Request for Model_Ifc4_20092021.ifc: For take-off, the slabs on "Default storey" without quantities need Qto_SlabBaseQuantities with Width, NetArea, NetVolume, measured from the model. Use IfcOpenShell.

First a look at what the model holds.

```python
import ifcopenshell
import ifcopenshell.util.element
import ifcopenshell.util.unit

model = ifcopenshell.open("Model_Ifc4_20092021.ifc")
print(model.schema)
for unit_type in ("LENGTHUNIT", "AREAUNIT", "VOLUMEUNIT"):
    print(unit_type, ifcopenshell.util.unit.calculate_unit_scale(model, unit_type))
storey = next(s for s in model.by_type("IfcBuildingStorey") if s.Name == "Default storey")
slabs = [e for e in ifcopenshell.util.element.get_decomposition(storey) if e.is_a("IfcSlab")]
for e in sorted(slabs, key=lambda e: e.id()):
    print(e.id(), e.is_a(), e.Name, list(ifcopenshell.util.element.get_psets(e, qtos_only=True)), sep=" | ")
```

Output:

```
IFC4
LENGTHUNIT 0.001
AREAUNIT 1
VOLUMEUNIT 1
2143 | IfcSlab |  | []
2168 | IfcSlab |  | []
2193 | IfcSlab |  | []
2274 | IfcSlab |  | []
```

```python
import ifcopenshell
import ifcopenshell.api.pset
import ifcopenshell.geom
import ifcopenshell.util.element
import ifcopenshell.util.shape
import ifcopenshell.util.unit

model = ifcopenshell.open("Model_Ifc4_20092021.ifc")
unit_scale = ifcopenshell.util.unit.calculate_unit_scale(model)
area_scale = ifcopenshell.util.unit.calculate_unit_scale(model, "AREAUNIT")
volume_scale = ifcopenshell.util.unit.calculate_unit_scale(model, "VOLUMEUNIT")
settings = ifcopenshell.geom.settings()

storey = next(s for s in model.by_type("IfcBuildingStorey") if s.Name == "Default storey")
slabs = [e for e in ifcopenshell.util.element.get_decomposition(storey) if e.is_a("IfcSlab")]

for e in sorted(slabs, key=lambda e: e.id()):
    if ifcopenshell.util.element.get_psets(e, qtos_only=True, should_inherit=False):
        continue
    # Geometry comes back in metres, in the element's own axes.
    shape = ifcopenshell.geom.create_shape(settings, e)
    values = {
        "Width": ifcopenshell.util.shape.get_z(shape.geometry) / unit_scale,
        "NetArea": ifcopenshell.util.shape.get_footprint_area(shape.geometry) / area_scale,
        "NetVolume": ifcopenshell.util.shape.get_volume(shape.geometry) / volume_scale,
    }
    qto = ifcopenshell.api.pset.add_qto(model, product=e, name="Qto_SlabBaseQuantities")
    ifcopenshell.api.pset.edit_qto(model, qto=qto, properties=values)
    print(e.id(), {k: round(v, 3) for k, v in values.items()})

model.write("Model_Ifc4_20092021_edited.ifc")
```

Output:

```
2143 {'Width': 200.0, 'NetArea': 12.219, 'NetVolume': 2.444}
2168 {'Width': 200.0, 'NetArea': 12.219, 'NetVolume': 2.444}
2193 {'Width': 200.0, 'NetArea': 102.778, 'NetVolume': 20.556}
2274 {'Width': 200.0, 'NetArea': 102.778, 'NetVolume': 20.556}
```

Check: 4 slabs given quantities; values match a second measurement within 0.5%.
